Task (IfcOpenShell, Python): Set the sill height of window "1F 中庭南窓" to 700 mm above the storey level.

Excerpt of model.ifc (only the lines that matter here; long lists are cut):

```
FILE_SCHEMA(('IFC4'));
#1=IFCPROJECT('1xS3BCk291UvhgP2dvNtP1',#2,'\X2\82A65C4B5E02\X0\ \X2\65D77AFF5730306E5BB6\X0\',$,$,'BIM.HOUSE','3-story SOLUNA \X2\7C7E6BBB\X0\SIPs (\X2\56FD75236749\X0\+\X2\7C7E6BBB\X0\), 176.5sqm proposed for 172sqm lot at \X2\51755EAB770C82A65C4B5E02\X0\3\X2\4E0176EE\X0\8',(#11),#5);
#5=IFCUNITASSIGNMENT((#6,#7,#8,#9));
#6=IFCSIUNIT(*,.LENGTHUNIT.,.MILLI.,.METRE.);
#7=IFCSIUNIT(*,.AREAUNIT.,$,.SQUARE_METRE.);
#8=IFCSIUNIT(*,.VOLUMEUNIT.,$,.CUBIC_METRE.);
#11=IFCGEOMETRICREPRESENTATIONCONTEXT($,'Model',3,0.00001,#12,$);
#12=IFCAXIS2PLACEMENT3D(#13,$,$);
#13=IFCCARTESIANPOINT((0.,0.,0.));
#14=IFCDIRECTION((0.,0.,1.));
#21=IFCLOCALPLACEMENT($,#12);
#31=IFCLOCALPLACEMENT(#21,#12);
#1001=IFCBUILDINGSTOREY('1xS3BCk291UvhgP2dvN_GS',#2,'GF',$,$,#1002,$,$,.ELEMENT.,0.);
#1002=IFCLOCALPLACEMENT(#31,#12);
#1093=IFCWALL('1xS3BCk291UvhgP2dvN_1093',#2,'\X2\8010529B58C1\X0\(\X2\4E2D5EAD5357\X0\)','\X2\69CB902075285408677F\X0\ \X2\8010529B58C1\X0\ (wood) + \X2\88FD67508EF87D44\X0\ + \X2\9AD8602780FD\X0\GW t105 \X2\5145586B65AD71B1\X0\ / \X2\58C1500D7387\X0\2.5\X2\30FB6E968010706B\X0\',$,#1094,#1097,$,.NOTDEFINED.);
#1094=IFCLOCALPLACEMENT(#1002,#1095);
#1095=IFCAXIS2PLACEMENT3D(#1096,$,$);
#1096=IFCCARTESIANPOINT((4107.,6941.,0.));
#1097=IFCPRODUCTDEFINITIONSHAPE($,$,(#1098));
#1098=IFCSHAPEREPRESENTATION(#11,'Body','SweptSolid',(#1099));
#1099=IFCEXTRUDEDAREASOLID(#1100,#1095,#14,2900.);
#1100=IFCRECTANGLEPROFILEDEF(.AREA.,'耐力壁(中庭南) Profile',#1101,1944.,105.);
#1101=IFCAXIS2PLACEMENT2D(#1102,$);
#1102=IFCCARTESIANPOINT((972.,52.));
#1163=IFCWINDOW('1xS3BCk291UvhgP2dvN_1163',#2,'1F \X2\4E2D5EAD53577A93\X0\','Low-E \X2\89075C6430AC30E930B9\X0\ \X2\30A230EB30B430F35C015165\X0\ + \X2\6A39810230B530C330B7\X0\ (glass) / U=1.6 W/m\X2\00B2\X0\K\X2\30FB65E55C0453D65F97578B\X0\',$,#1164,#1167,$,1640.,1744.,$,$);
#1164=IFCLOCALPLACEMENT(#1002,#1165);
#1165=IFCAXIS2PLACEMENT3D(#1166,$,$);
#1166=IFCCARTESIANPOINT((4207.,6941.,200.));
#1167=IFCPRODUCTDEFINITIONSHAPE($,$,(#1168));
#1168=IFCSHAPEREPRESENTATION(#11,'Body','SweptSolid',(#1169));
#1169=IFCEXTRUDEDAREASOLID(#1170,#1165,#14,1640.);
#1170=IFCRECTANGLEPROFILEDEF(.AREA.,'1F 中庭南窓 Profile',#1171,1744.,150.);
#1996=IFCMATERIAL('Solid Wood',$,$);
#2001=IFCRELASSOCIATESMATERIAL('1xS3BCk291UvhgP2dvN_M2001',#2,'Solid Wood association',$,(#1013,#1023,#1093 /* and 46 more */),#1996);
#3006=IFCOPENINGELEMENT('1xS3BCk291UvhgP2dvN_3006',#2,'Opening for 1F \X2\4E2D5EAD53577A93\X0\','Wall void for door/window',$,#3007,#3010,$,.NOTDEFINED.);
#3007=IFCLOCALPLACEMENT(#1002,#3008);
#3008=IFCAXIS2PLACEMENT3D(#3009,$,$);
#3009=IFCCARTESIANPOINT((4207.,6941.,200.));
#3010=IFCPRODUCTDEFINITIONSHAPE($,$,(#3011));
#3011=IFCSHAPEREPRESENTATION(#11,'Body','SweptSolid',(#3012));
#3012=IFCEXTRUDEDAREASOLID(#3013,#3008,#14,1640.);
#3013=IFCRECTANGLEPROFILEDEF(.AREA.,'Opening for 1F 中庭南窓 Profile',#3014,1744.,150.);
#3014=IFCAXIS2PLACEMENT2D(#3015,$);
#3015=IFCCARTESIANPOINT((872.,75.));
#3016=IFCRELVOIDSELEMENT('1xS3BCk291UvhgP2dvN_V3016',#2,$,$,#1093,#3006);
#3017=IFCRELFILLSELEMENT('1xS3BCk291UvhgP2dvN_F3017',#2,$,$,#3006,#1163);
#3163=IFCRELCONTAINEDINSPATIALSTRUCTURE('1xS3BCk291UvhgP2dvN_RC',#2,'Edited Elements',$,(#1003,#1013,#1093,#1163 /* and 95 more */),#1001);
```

```python
import numpy as np
import ifcopenshell
import ifcopenshell.api.geometry
import ifcopenshell.geom
import ifcopenshell.util.element
import ifcopenshell.util.placement
import ifcopenshell.util.shape
import ifcopenshell.util.unit

model = ifcopenshell.open("model.ifc")
unit_scale = ifcopenshell.util.unit.calculate_unit_scale(model)

window = model.by_guid("1xS3BCk291UvhgP2dvN_1163")
opening = window.FillsVoids[0].RelatingOpeningElement
storey = ifcopenshell.util.element.get_container(window, ifc_class="IfcBuildingStorey")
level = ifcopenshell.util.placement.get_local_placement(storey.ObjectPlacement)[2, 3]

# The opening's origin need not be at the sill, so measure its lowest point.
shape = ifcopenshell.geom.create_shape(ifcopenshell.geom.settings(), opening)
bottom = ifcopenshell.util.shape.get_shape_bottom_elevation(shape, shape.geometry) / unit_scale
dz = level + 0.7 / unit_scale - bottom

shift = np.array([0.0, 0.0, dz])
# The window is not placed relative to its opening, so move both.
for product in (opening, window):
    matrix = ifcopenshell.util.placement.get_local_placement(product.ObjectPlacement)
    matrix[:3, 3] += shift
    ifcopenshell.api.geometry.edit_object_placement(model, product=product, matrix=matrix, is_si=False)

print(f"moved by {dz * unit_scale:+.3f} m")

model.write("model-out.ifc")
```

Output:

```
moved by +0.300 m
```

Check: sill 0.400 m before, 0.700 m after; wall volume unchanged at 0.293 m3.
